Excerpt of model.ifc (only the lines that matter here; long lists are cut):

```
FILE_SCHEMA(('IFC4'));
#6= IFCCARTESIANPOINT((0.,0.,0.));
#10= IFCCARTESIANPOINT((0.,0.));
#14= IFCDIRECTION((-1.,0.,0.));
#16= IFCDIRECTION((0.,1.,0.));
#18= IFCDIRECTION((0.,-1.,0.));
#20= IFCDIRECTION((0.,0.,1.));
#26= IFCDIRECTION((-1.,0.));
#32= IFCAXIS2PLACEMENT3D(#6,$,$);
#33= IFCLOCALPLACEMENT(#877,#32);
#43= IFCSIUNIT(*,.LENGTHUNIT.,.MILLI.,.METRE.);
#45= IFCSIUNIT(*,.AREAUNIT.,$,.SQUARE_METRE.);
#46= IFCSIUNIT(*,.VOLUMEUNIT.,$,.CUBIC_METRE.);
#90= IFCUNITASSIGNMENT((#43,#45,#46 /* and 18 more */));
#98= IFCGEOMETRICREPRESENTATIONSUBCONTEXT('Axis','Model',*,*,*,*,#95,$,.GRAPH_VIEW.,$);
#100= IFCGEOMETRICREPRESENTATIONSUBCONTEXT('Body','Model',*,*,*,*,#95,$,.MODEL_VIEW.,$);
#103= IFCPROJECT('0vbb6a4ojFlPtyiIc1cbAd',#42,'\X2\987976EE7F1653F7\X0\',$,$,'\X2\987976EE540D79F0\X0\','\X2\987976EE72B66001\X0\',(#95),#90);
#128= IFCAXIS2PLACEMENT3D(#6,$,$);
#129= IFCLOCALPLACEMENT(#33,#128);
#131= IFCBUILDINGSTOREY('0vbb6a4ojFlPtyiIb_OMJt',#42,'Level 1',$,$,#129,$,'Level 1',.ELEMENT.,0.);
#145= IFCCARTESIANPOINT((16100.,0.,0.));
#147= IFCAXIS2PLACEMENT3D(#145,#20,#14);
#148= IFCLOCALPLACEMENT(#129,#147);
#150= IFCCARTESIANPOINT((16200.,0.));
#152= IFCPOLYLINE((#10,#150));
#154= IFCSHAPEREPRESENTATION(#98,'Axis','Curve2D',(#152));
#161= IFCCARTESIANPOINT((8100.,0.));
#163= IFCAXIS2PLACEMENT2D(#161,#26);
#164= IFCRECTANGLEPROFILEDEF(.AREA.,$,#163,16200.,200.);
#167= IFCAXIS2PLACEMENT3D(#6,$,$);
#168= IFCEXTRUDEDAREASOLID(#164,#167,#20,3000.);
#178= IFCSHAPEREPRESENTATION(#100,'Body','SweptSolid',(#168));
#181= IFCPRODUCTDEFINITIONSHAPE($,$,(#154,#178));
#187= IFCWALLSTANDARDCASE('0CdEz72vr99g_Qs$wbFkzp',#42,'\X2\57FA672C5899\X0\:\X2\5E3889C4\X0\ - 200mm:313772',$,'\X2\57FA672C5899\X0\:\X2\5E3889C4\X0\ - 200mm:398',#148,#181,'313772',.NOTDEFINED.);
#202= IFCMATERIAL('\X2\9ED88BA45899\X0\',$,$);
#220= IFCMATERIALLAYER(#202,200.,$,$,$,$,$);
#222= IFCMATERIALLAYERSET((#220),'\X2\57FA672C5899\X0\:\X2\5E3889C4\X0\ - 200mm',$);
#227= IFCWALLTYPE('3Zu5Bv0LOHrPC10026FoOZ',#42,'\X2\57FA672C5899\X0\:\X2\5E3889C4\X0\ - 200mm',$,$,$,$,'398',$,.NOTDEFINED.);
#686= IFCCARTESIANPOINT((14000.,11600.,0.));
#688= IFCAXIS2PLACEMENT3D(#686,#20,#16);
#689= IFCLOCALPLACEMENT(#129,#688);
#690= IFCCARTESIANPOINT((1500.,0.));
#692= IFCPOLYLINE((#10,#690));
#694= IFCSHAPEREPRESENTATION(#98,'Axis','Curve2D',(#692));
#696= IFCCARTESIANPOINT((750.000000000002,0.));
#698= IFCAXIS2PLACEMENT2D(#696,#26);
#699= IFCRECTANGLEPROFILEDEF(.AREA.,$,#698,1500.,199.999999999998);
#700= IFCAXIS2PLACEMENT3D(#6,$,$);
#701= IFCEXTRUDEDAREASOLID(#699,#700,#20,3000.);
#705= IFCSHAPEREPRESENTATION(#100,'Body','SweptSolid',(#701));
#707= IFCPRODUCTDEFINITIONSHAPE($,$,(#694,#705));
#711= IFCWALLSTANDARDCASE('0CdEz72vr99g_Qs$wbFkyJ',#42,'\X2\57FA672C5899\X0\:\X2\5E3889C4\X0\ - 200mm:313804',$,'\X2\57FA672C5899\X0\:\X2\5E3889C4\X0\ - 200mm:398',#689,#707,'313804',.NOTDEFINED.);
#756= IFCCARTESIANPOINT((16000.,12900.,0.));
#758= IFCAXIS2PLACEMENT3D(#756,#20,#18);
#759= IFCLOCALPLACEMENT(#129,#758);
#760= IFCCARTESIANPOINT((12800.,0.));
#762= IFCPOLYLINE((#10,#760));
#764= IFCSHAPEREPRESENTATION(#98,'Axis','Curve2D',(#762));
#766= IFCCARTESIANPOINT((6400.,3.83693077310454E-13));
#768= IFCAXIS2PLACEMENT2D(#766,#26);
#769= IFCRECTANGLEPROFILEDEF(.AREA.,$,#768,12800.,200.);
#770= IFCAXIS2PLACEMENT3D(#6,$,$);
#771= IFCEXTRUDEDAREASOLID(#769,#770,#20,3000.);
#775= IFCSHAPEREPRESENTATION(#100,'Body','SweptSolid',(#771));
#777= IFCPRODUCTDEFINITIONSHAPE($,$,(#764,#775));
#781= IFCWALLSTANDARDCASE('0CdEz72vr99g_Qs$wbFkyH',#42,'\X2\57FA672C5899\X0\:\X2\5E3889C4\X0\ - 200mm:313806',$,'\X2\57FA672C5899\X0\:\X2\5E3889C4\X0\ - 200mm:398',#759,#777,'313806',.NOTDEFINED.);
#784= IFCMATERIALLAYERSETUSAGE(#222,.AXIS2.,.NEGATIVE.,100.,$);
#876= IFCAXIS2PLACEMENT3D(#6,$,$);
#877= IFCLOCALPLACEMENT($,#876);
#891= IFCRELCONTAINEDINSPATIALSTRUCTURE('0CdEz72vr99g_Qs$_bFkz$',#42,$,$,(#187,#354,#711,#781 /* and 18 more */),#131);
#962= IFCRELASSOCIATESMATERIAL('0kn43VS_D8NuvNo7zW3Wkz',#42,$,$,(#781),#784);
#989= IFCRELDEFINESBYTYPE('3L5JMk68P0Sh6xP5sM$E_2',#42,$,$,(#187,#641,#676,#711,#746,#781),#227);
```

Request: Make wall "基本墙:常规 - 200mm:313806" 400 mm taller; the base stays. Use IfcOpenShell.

```python
import ifcopenshell
import ifcopenshell.geom
import ifcopenshell.util.representation
import ifcopenshell.util.shape
import ifcopenshell.util.unit

model = ifcopenshell.open("model.ifc")
unit_scale = ifcopenshell.util.unit.calculate_unit_scale(model)
settings = ifcopenshell.geom.settings()


def volume(element):
    """Net volume in cubic metres, openings subtracted."""
    shape = ifcopenshell.geom.create_shape(settings, element)
    return ifcopenshell.util.shape.get_volume(shape.geometry)


wall = model.by_guid("0CdEz72vr99g_Qs$wbFkyH")
before = volume(wall)

body = ifcopenshell.util.representation.get_representation(wall, "Model", "Body")
solid = body.Items[0]
old_height = solid.Depth
solid.Depth += 0.4 / unit_scale
after = volume(wall)

print(f"height {old_height:g} -> {solid.Depth:g}, volume {before:.3f} -> {after:.3f} m3")

model.write("model_rev.ifc")
```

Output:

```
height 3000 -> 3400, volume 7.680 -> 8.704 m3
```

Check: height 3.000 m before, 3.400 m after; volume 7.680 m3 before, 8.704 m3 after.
